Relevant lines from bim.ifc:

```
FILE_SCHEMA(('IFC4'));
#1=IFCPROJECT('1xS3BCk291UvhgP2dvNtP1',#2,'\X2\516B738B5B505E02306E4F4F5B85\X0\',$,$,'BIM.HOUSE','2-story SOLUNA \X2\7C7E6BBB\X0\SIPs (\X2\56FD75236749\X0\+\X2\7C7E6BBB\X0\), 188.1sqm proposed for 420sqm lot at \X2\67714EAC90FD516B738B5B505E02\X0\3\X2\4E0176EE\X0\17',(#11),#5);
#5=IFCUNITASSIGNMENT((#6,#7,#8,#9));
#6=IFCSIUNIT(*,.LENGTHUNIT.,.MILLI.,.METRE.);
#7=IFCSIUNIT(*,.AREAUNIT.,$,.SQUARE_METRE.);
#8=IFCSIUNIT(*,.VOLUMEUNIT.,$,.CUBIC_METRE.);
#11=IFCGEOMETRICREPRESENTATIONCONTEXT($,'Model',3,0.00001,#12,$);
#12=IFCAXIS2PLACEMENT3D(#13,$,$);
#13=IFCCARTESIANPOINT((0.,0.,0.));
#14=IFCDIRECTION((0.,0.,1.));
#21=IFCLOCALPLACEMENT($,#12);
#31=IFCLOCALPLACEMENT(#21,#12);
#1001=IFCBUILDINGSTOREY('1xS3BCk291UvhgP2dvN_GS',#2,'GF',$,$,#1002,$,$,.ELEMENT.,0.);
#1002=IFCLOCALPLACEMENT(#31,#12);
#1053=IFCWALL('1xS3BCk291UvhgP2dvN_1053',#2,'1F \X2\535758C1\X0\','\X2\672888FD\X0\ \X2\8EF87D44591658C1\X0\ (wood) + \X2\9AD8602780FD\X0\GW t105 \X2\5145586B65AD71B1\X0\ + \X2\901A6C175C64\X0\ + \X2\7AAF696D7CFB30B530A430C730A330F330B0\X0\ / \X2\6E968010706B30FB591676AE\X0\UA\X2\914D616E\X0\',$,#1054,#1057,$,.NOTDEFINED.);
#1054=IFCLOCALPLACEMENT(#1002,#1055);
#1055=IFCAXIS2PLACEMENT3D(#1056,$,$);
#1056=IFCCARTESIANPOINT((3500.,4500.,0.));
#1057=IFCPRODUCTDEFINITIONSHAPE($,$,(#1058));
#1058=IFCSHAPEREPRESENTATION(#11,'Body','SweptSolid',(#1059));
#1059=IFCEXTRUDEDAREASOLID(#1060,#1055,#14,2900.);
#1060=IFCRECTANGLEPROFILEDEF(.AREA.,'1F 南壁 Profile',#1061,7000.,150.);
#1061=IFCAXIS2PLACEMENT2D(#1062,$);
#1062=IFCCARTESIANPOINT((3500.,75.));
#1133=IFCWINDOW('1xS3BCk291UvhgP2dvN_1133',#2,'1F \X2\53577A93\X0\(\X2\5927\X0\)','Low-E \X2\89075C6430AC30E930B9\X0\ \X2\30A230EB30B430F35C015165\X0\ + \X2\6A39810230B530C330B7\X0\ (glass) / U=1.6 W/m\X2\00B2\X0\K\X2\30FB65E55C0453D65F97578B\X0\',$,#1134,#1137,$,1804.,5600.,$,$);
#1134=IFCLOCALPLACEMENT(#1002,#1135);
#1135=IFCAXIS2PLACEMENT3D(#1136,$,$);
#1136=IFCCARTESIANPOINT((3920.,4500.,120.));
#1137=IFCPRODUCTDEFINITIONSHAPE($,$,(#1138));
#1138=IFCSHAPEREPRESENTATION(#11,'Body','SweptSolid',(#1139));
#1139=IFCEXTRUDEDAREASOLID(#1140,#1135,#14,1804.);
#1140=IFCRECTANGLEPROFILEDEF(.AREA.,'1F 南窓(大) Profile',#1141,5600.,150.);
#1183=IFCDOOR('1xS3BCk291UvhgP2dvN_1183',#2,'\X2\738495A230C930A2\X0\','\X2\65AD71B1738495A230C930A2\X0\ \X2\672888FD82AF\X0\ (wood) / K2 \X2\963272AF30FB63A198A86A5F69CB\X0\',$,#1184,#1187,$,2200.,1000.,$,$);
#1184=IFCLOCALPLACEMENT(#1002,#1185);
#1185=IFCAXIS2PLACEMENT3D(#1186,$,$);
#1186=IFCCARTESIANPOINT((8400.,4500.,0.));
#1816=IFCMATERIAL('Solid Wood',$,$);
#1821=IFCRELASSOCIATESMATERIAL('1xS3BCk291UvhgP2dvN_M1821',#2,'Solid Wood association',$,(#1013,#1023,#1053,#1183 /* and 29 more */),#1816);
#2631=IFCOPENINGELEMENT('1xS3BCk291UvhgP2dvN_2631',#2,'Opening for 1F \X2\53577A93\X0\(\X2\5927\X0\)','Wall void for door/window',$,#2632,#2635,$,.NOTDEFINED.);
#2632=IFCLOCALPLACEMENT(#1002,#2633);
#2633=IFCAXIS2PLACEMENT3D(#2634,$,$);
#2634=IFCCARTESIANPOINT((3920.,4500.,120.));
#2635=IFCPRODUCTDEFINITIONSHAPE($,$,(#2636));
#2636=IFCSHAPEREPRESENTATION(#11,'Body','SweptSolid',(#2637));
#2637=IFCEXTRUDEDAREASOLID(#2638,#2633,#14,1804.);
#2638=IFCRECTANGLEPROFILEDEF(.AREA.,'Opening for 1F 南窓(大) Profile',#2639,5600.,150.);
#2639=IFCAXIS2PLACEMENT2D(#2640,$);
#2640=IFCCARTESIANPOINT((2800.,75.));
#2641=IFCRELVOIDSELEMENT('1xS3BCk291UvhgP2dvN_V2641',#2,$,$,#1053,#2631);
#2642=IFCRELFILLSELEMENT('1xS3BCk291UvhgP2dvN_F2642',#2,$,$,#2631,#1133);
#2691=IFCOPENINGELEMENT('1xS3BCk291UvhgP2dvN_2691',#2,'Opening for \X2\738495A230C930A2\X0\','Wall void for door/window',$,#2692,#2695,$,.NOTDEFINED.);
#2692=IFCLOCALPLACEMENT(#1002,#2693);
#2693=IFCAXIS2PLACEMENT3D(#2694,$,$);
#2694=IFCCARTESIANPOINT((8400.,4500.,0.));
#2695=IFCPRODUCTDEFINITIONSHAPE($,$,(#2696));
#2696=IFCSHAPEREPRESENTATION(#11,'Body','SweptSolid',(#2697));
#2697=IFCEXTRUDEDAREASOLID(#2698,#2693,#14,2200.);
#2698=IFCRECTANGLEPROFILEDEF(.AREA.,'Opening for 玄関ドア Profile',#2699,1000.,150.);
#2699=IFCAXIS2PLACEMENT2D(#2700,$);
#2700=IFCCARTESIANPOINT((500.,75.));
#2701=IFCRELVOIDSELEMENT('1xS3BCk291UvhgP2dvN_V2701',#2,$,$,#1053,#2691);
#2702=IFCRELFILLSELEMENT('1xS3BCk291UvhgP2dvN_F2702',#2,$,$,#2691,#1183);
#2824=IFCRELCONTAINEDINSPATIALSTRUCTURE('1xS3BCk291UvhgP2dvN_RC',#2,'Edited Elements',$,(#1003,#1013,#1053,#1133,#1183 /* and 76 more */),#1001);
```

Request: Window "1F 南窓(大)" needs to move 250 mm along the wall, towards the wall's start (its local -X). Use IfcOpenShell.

```python
import ifcopenshell
import ifcopenshell.api.geometry
import ifcopenshell.util.placement

model = ifcopenshell.open("bim.ifc")

window = model.by_id(1133)
opening = window.FillsVoids[0].RelatingOpeningElement
wall = opening.VoidsElements[0].RelatingBuildingElement

wall_matrix = ifcopenshell.util.placement.get_local_placement(wall.ObjectPlacement)
shift = wall_matrix[:3, 0] * -250.0
before = ifcopenshell.util.placement.get_local_placement(window.ObjectPlacement)[:3, 3].copy()

# The window is not placed relative to its opening, so move both.
for product in (opening, window):
    matrix = ifcopenshell.util.placement.get_local_placement(product.ObjectPlacement)
    matrix[:3, 3] += shift
    ifcopenshell.api.geometry.edit_object_placement(model, product=product, matrix=matrix, is_si=False)

after = ifcopenshell.util.placement.get_local_placement(window.ObjectPlacement)[:3, 3]
print("window moved by", (after - before).round(3) + 0.0)

model.write("bim_rev.ifc")
```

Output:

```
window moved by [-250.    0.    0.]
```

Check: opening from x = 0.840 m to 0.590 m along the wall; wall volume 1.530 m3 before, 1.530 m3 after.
